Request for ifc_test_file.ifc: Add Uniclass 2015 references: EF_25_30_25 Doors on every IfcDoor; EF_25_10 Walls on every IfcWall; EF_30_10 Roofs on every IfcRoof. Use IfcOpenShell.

First a look at what the model holds.

```python
import ifcopenshell

model = ifcopenshell.open("ifc_test_file.ifc")
print(model.schema)
print("classifications:", [c.Name for c in model.by_type("IfcClassification")])
for ifc_class in ("IfcDoor", "IfcRoof", "IfcStair", "IfcWall", "IfcWindow"):
    print(ifc_class, len(model.by_type(ifc_class)))
```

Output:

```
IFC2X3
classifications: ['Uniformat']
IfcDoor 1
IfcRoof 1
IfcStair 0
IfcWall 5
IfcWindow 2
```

```python
import ifcopenshell
import ifcopenshell.api.classification

model = ifcopenshell.open("ifc_test_file.ifc")

# IFC2X3 requires Source and Edition and has no link from the project to the system.
system = model.create_entity("IfcClassification", Source="NBS", Edition="2015", Name="Uniclass 2015")

codes = {
    "IfcDoor": ("EF_25_30_25", "Doors"),
    "IfcWall": ("EF_25_10", "Walls"),
    "IfcRoof": ("EF_30_10", "Roofs"),
}
for ifc_class, (code, name) in codes.items():
    products = model.by_type(ifc_class)
    ifcopenshell.api.classification.add_reference(
        model, products=products, classification=system, identification=code, name=name
    )
    print(code, len(products))

model.write("ifc_test_file_updated.ifc")
```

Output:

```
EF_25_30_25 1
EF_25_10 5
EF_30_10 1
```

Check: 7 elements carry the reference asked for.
